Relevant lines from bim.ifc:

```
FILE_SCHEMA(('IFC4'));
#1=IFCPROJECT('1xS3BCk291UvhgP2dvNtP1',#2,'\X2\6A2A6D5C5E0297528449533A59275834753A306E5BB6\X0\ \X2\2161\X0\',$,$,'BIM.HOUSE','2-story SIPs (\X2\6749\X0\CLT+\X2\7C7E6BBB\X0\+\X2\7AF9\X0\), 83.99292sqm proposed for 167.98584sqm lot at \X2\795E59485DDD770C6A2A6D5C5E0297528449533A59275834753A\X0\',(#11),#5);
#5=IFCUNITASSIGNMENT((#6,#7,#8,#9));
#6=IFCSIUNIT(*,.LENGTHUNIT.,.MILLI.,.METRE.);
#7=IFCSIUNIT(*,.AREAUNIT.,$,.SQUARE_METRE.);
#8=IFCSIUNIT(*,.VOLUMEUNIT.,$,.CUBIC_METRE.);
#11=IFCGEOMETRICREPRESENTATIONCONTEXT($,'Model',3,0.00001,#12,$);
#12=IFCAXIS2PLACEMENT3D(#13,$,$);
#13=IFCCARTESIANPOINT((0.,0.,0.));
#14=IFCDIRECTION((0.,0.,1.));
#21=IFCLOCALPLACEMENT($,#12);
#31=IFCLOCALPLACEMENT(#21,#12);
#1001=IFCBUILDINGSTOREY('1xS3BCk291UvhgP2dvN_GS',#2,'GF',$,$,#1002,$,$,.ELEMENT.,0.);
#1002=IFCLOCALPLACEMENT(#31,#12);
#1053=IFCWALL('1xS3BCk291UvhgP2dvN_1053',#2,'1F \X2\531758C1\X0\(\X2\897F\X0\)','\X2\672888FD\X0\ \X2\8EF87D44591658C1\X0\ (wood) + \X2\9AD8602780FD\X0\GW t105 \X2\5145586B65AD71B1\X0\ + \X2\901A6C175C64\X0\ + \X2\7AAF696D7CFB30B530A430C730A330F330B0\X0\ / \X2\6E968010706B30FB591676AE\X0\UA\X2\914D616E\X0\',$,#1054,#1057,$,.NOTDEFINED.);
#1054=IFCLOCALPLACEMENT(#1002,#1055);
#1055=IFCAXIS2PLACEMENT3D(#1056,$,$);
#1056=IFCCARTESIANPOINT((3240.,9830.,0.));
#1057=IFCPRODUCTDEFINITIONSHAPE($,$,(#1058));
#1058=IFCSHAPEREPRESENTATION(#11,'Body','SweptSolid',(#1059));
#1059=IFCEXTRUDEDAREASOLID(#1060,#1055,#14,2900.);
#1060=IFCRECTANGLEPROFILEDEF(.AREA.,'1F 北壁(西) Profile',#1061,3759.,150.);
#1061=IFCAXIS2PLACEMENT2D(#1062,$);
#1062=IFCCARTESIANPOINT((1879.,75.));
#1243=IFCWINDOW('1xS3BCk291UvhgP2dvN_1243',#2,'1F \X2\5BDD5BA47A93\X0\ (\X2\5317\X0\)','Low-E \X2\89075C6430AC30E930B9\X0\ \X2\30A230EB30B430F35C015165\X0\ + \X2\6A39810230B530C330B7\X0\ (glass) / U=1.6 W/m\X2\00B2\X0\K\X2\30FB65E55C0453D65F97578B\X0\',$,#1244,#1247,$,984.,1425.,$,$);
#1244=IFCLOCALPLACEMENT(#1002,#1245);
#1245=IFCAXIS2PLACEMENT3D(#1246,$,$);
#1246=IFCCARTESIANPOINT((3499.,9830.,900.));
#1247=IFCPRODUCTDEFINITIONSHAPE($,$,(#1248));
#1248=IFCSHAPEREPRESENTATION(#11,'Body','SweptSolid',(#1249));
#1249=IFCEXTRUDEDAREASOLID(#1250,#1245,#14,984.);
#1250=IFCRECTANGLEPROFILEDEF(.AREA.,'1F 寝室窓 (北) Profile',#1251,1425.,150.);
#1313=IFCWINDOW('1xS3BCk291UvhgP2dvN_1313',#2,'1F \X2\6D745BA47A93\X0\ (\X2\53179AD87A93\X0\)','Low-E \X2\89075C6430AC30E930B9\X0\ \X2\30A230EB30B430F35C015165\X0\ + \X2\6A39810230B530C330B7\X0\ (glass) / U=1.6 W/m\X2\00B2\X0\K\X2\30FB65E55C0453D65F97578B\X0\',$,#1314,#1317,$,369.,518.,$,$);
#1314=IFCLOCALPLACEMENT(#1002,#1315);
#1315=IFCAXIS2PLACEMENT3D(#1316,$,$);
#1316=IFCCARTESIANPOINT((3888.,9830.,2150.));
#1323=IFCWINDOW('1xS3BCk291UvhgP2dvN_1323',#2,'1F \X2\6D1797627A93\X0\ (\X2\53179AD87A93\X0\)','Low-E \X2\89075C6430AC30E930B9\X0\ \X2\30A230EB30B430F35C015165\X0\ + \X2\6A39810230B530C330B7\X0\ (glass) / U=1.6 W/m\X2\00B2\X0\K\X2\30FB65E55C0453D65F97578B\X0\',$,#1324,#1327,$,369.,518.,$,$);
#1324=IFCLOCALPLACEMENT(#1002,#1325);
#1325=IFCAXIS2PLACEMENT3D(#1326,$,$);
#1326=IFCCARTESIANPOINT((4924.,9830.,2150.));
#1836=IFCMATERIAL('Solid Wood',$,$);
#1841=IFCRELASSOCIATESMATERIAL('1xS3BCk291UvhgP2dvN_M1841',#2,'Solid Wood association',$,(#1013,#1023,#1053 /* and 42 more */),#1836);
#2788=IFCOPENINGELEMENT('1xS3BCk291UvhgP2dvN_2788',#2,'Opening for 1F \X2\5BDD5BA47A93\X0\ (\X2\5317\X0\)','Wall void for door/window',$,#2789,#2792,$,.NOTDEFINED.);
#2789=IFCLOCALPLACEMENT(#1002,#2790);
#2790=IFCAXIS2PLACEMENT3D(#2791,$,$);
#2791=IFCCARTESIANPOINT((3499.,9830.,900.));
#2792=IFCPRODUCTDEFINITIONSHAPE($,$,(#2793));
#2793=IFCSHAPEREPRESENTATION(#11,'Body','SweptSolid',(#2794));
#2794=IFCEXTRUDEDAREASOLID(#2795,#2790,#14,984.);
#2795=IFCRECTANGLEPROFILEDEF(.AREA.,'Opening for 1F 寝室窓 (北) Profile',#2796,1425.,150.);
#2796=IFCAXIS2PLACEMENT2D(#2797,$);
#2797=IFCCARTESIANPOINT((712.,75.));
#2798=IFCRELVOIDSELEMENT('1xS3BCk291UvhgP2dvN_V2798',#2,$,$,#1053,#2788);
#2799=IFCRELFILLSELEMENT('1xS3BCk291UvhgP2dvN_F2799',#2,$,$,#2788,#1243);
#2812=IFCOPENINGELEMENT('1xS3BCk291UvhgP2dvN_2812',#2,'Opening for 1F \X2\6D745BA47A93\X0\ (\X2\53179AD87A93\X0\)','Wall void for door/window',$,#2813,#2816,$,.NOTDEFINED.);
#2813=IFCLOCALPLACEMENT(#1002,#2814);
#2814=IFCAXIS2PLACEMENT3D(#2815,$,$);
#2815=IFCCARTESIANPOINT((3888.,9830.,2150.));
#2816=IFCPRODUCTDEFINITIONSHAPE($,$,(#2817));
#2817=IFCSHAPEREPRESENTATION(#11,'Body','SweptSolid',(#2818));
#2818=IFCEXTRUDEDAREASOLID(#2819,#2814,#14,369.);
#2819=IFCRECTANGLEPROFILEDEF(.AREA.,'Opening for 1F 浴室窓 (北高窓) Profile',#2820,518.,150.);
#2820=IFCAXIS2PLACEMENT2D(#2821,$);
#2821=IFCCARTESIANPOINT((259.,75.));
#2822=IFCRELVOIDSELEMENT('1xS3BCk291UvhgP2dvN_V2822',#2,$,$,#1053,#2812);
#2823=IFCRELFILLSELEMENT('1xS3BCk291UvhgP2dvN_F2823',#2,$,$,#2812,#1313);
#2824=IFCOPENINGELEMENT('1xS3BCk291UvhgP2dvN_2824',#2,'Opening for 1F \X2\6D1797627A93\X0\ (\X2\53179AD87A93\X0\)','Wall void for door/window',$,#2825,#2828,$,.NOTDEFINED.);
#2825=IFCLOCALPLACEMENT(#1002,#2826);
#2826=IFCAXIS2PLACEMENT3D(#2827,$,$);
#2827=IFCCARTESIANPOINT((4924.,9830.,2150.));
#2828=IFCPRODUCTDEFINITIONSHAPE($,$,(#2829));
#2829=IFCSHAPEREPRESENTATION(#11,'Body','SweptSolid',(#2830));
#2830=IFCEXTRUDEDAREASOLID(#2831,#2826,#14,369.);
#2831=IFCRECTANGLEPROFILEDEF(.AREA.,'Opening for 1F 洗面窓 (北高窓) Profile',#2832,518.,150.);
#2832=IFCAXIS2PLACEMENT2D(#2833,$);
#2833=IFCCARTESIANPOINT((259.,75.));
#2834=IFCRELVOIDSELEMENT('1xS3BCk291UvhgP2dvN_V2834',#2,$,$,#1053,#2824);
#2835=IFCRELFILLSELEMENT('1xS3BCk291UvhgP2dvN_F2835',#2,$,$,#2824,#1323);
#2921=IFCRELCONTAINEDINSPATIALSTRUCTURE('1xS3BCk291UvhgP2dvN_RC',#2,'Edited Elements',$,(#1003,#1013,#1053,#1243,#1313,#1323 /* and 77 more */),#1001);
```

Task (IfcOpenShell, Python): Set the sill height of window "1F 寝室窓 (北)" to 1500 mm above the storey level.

```python
import numpy as np
import ifcopenshell
import ifcopenshell.api.geometry
import ifcopenshell.geom
import ifcopenshell.util.element
import ifcopenshell.util.placement
import ifcopenshell.util.shape
import ifcopenshell.util.unit

model = ifcopenshell.open("bim.ifc")
unit_scale = ifcopenshell.util.unit.calculate_unit_scale(model)

window = model.by_id(1243)
opening = window.FillsVoids[0].RelatingOpeningElement
storey = ifcopenshell.util.element.get_container(window, ifc_class="IfcBuildingStorey")
level = ifcopenshell.util.placement.get_local_placement(storey.ObjectPlacement)[2, 3]

# The opening's origin need not be at the sill, so measure its lowest point.
shape = ifcopenshell.geom.create_shape(ifcopenshell.geom.settings(), opening)
bottom = ifcopenshell.util.shape.get_shape_bottom_elevation(shape, shape.geometry) / unit_scale
dz = level + 1.5 / unit_scale - bottom

shift = np.array([0.0, 0.0, dz])
# The window is not placed relative to its opening, so move both.
for product in (opening, window):
    matrix = ifcopenshell.util.placement.get_local_placement(product.ObjectPlacement)
    matrix[:3, 3] += shift
    ifcopenshell.api.geometry.edit_object_placement(model, product=product, matrix=matrix, is_si=False)

print(f"moved by {dz * unit_scale:+.3f} m")

model.write("bim_rev.ifc")
```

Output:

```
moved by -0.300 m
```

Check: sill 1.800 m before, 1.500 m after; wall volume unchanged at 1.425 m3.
